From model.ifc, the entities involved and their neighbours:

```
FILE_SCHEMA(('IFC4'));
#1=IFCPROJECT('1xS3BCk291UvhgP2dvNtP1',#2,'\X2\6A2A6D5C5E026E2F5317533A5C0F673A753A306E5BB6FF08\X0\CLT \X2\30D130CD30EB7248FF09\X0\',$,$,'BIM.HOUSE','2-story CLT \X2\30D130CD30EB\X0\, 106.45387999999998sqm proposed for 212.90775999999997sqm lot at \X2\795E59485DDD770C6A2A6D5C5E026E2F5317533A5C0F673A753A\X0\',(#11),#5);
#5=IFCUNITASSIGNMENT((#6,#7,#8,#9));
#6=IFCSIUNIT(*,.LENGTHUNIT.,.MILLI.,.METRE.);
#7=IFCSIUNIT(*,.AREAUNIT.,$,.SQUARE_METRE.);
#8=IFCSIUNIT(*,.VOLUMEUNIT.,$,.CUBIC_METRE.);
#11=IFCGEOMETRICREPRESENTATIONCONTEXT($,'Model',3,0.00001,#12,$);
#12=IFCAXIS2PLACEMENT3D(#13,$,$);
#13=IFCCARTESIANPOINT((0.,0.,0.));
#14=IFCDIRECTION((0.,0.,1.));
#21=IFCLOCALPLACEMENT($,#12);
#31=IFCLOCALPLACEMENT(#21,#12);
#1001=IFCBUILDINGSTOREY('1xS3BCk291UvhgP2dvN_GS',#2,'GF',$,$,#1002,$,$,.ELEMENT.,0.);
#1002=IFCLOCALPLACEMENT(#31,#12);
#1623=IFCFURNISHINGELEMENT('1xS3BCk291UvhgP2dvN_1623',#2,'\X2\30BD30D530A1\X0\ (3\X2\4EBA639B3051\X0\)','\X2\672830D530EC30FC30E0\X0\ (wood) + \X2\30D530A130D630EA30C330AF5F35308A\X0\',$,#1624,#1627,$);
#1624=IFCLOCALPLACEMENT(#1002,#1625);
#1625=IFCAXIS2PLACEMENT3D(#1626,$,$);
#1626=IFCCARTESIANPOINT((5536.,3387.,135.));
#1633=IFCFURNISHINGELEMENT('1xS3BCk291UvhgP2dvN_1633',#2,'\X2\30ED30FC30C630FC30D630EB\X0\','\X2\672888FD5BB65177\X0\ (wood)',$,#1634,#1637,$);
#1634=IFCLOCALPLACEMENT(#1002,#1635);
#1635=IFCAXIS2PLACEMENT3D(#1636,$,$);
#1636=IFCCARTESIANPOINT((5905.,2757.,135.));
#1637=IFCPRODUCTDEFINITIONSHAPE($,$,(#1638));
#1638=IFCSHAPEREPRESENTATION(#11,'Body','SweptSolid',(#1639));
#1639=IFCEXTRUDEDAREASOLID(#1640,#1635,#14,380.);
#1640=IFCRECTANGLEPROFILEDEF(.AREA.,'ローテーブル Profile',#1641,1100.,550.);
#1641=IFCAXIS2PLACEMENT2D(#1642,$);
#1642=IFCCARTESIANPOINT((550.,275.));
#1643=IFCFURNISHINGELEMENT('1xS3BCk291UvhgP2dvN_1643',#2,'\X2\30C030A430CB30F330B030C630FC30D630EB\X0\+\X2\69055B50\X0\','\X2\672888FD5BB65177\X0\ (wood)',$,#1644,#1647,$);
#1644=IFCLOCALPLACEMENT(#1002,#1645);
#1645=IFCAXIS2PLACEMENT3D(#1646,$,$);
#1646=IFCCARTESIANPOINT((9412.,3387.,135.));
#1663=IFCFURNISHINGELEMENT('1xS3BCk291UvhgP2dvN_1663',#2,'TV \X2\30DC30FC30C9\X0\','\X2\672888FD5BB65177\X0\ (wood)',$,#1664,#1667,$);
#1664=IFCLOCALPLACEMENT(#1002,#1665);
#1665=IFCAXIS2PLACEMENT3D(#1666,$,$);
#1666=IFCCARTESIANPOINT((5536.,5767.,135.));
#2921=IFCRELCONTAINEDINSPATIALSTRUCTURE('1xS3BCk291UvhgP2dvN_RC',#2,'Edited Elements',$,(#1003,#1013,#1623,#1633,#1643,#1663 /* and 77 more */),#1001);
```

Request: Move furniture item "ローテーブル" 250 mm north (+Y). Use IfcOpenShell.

```python
import ifcopenshell
import ifcopenshell.api.geometry
import ifcopenshell.util.placement

model = ifcopenshell.open("model.ifc")

item = model.by_guid("1xS3BCk291UvhgP2dvN_1633")
matrix = ifcopenshell.util.placement.get_local_placement(item.ObjectPlacement)
matrix[1, 3] += 250.0
ifcopenshell.api.geometry.edit_object_placement(model, product=item, matrix=matrix, is_si=False)

print(ifcopenshell.util.placement.get_local_placement(item.ObjectPlacement).round(3) + 0.0)

model.write("model_edited.ifc")
```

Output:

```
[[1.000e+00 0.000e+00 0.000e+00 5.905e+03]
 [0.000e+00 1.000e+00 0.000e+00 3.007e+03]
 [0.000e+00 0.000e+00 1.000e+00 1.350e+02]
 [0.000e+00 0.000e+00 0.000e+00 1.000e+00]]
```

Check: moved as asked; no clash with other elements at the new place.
